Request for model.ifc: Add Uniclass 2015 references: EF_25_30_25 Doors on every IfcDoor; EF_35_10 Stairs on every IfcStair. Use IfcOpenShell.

First a look at what the model holds.

```python
import ifcopenshell

model = ifcopenshell.open("model.ifc")
print(model.schema)
print("classifications:", [c.Name for c in model.by_type("IfcClassification")])
for ifc_class in ("IfcDoor", "IfcRoof", "IfcStair", "IfcWall", "IfcWindow"):
    print(ifc_class, len(model.by_type(ifc_class)))
```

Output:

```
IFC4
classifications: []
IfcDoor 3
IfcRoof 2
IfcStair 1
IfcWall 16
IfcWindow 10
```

```python
import ifcopenshell
import ifcopenshell.api.classification

model = ifcopenshell.open("model.ifc")

system = ifcopenshell.api.classification.add_classification(model, classification="Uniclass 2015")

codes = {
    "IfcDoor": ("EF_25_30_25", "Doors"),
    "IfcStair": ("EF_35_10", "Stairs"),
}
for ifc_class, (code, name) in codes.items():
    products = model.by_type(ifc_class)
    ifcopenshell.api.classification.add_reference(
        model, products=products, classification=system, identification=code, name=name
    )
    print(code, len(products))

model.write("model_rev.ifc")
```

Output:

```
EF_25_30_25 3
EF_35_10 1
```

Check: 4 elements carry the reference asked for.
